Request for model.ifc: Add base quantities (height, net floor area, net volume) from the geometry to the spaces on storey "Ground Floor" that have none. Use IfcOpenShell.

First a look at what the model holds.

```python
import ifcopenshell
import ifcopenshell.util.element
import ifcopenshell.util.unit

model = ifcopenshell.open("model.ifc")
print(model.schema)
for unit_type in ("LENGTHUNIT", "AREAUNIT", "VOLUMEUNIT"):
    print(unit_type, ifcopenshell.util.unit.calculate_unit_scale(model, unit_type))
storey = next(s for s in model.by_type("IfcBuildingStorey") if s.Name == "Ground Floor")
spaces = [e for e in ifcopenshell.util.element.get_decomposition(storey) if e.is_a("IfcSpace")]
for e in sorted(spaces, key=lambda e: e.id()):
    print(e.id(), e.is_a(), e.Name, list(ifcopenshell.util.element.get_psets(e, qtos_only=True)), sep=" | ")
```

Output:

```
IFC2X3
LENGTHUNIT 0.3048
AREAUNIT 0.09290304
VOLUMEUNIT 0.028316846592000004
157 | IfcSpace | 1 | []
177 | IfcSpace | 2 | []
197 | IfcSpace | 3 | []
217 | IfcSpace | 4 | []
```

```python
import ifcopenshell
import ifcopenshell.api.pset
import ifcopenshell.geom
import ifcopenshell.util.element
import ifcopenshell.util.shape
import ifcopenshell.util.unit

model = ifcopenshell.open("model.ifc")
unit_scale = ifcopenshell.util.unit.calculate_unit_scale(model)
area_scale = ifcopenshell.util.unit.calculate_unit_scale(model, "AREAUNIT")
volume_scale = ifcopenshell.util.unit.calculate_unit_scale(model, "VOLUMEUNIT")
settings = ifcopenshell.geom.settings()

storey = next(s for s in model.by_type("IfcBuildingStorey") if s.Name == "Ground Floor")
spaces = [e for e in ifcopenshell.util.element.get_decomposition(storey) if e.is_a("IfcSpace")]

for e in sorted(spaces, key=lambda e: e.id()):
    if ifcopenshell.util.element.get_psets(e, qtos_only=True, should_inherit=False):
        continue
    # Geometry comes back in metres, in the element's own axes.
    shape = ifcopenshell.geom.create_shape(settings, e)
    values = {
        "Height": ifcopenshell.util.shape.get_z(shape.geometry) / unit_scale,
        "NetFloorArea": ifcopenshell.util.shape.get_footprint_area(shape.geometry) / area_scale,
        "NetVolume": ifcopenshell.util.shape.get_volume(shape.geometry) / volume_scale,
    }
    qto = ifcopenshell.api.pset.add_qto(model, product=e, name="BaseQuantities")
    ifcopenshell.api.pset.edit_qto(model, qto=qto, properties=values)
    print(e.id(), {k: round(v, 3) for k, v in values.items()})

model.write("model_edited.ifc")
```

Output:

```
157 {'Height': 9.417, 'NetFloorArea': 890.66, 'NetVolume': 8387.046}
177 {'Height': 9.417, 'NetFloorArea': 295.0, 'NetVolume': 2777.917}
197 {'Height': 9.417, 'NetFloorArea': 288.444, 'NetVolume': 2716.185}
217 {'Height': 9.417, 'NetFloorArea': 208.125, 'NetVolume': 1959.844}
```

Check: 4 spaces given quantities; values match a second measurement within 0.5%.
